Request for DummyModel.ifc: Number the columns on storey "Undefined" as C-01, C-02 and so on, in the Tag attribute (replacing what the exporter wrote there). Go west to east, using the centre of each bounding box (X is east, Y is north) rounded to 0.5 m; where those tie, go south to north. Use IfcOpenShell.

First a look at what the model holds.

```python
import ifcopenshell
import ifcopenshell.util.element
import ifcopenshell.util.placement

model = ifcopenshell.open("DummyModel.ifc")
print(model.schema)
storey = next(s for s in model.by_type("IfcBuildingStorey") if s.Name == "Undefined")
columns = [e for e in ifcopenshell.util.element.get_decomposition(storey) if e.is_a("IfcColumn")]
for e in sorted(columns, key=lambda e: e.id()):
    origin = ifcopenshell.util.placement.get_local_placement(e.ObjectPlacement)[:3, 3]
    print(e.id(), e.Tag, e.Name, origin.round(2) + 0.0, sep=" | ")
```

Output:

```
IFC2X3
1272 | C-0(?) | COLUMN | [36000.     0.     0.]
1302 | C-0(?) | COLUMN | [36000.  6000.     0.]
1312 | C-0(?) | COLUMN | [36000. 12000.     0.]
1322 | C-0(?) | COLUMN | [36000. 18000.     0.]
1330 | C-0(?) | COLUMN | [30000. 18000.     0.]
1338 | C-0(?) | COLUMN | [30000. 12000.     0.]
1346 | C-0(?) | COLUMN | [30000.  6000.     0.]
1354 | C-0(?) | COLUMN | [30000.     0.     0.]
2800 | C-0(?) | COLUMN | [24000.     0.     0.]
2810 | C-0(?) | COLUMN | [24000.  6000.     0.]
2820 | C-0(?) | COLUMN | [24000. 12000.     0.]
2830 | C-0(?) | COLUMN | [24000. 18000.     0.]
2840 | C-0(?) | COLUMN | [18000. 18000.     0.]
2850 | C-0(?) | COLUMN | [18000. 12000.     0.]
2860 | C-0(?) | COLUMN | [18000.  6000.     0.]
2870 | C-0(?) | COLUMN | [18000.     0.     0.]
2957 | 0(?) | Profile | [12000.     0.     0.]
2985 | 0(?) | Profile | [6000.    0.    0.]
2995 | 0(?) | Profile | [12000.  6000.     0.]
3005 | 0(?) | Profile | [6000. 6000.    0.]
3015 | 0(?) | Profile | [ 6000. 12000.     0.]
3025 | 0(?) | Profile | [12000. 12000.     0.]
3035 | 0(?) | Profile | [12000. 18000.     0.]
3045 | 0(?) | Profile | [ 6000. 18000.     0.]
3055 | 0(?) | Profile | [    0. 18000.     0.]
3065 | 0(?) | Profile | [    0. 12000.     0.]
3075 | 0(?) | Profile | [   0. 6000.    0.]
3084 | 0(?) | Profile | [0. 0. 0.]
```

```python
import ifcopenshell
import ifcopenshell.geom
import ifcopenshell.util.element
import ifcopenshell.util.shape

model = ifcopenshell.open("DummyModel.ifc")
settings = ifcopenshell.geom.settings()
settings.set("use-world-coords", True)


def centre(element):
    shape = ifcopenshell.geom.create_shape(settings, element)
    return ifcopenshell.util.shape.get_bbox_centroid(shape.geometry)


storey = next(s for s in model.by_type("IfcBuildingStorey") if s.Name == "Undefined")
columns = [e for e in ifcopenshell.util.element.get_decomposition(storey) if e.is_a("IfcColumn")]

# Insertion points can sit at a corner or the storey origin, so sort by the geometry (in metres).
centres = {e: centre(e) for e in columns}
columns.sort(key=lambda e: (round(centres[e][0] / 0.5), centres[e][1]))

for i, e in enumerate(columns, start=1):
    number = f"C-{i:02d}"
    e.Tag = number
    print(e.id(), number)

model.write("DummyModel_edited.ifc")
```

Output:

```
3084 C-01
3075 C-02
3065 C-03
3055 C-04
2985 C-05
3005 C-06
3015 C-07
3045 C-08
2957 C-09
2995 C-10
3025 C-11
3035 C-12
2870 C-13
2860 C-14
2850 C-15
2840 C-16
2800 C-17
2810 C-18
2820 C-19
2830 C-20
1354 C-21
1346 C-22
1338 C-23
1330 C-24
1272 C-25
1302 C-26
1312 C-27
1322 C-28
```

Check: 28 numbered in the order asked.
